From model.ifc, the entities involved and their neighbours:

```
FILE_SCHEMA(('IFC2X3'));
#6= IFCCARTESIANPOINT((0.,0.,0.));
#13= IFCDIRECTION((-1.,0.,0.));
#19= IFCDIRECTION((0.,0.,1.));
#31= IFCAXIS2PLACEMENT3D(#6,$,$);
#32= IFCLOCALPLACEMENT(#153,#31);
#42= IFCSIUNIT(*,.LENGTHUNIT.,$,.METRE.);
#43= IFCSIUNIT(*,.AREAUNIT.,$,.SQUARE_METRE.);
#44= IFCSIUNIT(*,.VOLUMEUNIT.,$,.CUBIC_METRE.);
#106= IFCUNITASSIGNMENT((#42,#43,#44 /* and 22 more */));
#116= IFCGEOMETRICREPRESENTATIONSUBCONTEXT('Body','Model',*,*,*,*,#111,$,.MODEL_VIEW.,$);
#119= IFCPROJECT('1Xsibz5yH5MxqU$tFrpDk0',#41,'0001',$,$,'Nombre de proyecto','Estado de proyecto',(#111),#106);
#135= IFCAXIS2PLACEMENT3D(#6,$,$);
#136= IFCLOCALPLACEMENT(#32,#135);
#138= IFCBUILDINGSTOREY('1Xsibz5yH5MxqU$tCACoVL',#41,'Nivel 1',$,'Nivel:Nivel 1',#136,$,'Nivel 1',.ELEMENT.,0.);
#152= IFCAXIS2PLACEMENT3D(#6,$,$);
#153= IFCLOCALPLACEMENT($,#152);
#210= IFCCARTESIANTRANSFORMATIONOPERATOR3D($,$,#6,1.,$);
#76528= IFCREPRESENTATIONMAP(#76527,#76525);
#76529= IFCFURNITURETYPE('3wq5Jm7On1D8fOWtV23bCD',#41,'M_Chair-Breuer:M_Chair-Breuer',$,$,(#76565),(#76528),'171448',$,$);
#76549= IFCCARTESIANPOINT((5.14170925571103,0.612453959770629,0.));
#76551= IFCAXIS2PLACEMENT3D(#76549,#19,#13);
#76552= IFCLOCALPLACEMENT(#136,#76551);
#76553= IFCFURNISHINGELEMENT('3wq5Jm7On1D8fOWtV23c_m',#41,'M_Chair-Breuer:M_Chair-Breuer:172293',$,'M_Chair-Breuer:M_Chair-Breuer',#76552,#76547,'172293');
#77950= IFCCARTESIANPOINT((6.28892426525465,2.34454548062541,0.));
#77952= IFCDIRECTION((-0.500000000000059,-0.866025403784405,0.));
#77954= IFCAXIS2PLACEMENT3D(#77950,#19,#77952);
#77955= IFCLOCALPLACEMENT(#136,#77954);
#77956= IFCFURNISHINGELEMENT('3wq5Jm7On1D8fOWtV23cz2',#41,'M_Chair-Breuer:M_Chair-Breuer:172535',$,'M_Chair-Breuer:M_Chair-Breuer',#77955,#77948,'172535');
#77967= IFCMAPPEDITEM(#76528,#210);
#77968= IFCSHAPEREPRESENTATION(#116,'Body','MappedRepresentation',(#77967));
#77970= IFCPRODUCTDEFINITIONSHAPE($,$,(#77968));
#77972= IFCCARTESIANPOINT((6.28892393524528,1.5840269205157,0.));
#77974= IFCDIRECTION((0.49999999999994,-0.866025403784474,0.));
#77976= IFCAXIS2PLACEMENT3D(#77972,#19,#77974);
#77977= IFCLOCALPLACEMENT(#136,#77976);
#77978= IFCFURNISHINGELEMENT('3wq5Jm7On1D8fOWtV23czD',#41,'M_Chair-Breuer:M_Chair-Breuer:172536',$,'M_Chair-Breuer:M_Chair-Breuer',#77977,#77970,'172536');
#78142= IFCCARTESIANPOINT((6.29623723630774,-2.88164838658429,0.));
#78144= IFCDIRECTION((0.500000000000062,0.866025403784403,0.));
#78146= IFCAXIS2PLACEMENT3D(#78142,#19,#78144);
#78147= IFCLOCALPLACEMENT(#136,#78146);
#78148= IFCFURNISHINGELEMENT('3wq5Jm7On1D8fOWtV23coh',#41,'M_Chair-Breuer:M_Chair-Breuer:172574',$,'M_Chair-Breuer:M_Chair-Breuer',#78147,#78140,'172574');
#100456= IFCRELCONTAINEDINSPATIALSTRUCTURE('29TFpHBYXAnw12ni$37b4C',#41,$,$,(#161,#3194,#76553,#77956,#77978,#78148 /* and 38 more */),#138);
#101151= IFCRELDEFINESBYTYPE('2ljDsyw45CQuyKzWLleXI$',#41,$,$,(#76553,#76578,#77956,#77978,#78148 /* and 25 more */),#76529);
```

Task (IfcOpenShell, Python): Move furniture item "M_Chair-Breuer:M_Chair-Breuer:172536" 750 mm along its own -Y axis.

```python
import ifcopenshell
import ifcopenshell.api.geometry
import ifcopenshell.util.placement
import ifcopenshell.util.unit

model = ifcopenshell.open("model.ifc")
unit_scale = ifcopenshell.util.unit.calculate_unit_scale(model)

item = model.by_guid("3wq5Jm7On1D8fOWtV23czD")
matrix = ifcopenshell.util.placement.get_local_placement(item.ObjectPlacement)
matrix[:3, 3] -= matrix[:3, 1] * 0.75 / unit_scale
ifcopenshell.api.geometry.edit_object_placement(model, product=item, matrix=matrix, is_si=False)

print(ifcopenshell.util.placement.get_local_placement(item.ObjectPlacement).round(3) + 0.0)

model.write("model-out.ifc")
```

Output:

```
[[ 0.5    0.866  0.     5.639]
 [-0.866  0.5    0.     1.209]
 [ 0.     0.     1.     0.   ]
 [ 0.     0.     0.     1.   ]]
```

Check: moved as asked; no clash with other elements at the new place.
